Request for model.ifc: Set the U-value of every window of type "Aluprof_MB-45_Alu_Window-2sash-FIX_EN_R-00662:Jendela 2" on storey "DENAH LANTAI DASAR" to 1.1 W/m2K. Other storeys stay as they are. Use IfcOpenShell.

First a look at what the model holds.

```python
import ifcopenshell
import ifcopenshell.util.element

model = ifcopenshell.open("model.ifc")
print(model.schema)
storey = next(s for s in model.by_type("IfcBuildingStorey") if s.Name == "DENAH LANTAI DASAR")
windows = [e for e in ifcopenshell.util.element.get_decomposition(storey) if e.is_a("IfcWindow")]
seen = {}
for e in windows:
    element_type = ifcopenshell.util.element.get_type(e)
    key = (element_type.Name if element_type != e and element_type else None, ifcopenshell.util.element.get_pset(e, "Pset_WindowCommon", "ThermalTransmittance"))
    seen[key] = seen.get(key, 0) + 1
for (name, value), count in sorted(seen.items(), key=str):
    print(count, "x", name, "|", value)
```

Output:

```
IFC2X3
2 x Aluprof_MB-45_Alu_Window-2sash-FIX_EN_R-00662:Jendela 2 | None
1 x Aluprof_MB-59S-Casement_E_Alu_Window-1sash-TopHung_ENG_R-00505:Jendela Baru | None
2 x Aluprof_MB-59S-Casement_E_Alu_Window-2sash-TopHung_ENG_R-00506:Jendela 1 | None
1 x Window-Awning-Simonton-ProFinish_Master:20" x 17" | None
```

```python
import ifcopenshell
import ifcopenshell.api.pset
import ifcopenshell.util.element

model = ifcopenshell.open("model.ifc")

storey = next(s for s in model.by_type("IfcBuildingStorey") if s.Name == "DENAH LANTAI DASAR")
windows = [e for e in ifcopenshell.util.element.get_decomposition(storey) if e.is_a("IfcWindow")]

count = 0
for e in windows:
    element_type = ifcopenshell.util.element.get_type(e)
    if element_type in (None, e) or element_type.Name != "Aluprof_MB-45_Alu_Window-2sash-FIX_EN_R-00662:Jendela 2":
        continue
    # add_pset returns the element's existing set when there is one.
    pset = ifcopenshell.api.pset.add_pset(model, product=e, name="Pset_WindowCommon")
    ifcopenshell.api.pset.edit_pset(model, pset=pset, properties={"ThermalTransmittance": 1.1})
    count += 1

print(count, "windows updated")

model.write("model_updated.ifc")
```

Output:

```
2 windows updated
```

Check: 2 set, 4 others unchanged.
